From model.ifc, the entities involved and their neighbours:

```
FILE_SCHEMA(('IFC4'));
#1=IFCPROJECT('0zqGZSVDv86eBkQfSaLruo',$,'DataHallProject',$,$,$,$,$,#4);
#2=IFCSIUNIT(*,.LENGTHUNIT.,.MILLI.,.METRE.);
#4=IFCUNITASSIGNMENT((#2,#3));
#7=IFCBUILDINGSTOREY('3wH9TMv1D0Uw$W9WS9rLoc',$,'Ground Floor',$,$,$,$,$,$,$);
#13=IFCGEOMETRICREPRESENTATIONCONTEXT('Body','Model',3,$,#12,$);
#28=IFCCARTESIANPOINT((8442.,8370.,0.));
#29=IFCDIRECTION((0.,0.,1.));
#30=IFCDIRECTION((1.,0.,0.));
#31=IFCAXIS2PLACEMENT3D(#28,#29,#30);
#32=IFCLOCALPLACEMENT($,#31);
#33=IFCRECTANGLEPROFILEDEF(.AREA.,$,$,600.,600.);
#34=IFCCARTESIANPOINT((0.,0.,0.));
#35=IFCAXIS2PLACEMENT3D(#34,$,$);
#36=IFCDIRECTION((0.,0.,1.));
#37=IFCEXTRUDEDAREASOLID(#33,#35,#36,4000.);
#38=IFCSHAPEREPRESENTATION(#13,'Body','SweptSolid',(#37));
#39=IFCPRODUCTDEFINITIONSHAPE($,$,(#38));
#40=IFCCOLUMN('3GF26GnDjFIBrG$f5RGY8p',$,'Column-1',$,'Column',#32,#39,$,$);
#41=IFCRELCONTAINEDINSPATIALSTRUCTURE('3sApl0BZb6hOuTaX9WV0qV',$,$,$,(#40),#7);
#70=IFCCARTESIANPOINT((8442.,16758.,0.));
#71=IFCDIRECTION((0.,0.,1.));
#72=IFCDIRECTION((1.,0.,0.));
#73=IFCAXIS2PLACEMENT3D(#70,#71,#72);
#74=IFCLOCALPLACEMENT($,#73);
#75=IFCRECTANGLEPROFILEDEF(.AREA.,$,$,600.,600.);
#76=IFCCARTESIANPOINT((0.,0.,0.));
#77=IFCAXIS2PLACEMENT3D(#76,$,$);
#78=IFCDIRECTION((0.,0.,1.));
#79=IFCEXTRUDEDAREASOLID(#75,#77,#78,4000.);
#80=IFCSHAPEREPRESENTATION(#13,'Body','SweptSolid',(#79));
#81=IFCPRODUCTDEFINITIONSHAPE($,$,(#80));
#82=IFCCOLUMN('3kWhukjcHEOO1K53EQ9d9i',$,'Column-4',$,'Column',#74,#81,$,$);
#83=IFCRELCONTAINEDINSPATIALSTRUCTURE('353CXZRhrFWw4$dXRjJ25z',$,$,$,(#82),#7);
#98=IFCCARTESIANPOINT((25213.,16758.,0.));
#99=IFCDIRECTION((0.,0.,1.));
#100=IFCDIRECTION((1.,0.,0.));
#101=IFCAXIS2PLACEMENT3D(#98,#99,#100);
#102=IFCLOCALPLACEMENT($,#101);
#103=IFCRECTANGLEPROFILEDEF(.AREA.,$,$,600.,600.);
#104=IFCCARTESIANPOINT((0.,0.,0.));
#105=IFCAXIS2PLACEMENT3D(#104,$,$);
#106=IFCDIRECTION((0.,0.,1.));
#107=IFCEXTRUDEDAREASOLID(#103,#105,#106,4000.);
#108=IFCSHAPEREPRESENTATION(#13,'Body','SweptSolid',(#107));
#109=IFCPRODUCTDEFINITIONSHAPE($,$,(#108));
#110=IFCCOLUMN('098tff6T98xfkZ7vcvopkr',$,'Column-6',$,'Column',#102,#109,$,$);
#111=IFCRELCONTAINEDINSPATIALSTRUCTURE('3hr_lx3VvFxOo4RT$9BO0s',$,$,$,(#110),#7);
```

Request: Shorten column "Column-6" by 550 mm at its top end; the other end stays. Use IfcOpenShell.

```python
import ifcopenshell

model = ifcopenshell.open("model.ifc")

member = model.by_guid("098tff6T98xfkZ7vcvopkr")
change = -550.0

# The extrusion runs towards the end named, so only its depth changes.
body = next(r for r in member.Representation.Representations if r.RepresentationIdentifier == "Body")
solid = body.Items[0]
old_length = solid.Depth
solid.Depth += change

print(f"length {old_length:g} -> {solid.Depth:g}")

model.write("model_updated.ifc")
```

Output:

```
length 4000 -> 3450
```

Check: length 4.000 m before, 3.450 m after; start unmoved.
